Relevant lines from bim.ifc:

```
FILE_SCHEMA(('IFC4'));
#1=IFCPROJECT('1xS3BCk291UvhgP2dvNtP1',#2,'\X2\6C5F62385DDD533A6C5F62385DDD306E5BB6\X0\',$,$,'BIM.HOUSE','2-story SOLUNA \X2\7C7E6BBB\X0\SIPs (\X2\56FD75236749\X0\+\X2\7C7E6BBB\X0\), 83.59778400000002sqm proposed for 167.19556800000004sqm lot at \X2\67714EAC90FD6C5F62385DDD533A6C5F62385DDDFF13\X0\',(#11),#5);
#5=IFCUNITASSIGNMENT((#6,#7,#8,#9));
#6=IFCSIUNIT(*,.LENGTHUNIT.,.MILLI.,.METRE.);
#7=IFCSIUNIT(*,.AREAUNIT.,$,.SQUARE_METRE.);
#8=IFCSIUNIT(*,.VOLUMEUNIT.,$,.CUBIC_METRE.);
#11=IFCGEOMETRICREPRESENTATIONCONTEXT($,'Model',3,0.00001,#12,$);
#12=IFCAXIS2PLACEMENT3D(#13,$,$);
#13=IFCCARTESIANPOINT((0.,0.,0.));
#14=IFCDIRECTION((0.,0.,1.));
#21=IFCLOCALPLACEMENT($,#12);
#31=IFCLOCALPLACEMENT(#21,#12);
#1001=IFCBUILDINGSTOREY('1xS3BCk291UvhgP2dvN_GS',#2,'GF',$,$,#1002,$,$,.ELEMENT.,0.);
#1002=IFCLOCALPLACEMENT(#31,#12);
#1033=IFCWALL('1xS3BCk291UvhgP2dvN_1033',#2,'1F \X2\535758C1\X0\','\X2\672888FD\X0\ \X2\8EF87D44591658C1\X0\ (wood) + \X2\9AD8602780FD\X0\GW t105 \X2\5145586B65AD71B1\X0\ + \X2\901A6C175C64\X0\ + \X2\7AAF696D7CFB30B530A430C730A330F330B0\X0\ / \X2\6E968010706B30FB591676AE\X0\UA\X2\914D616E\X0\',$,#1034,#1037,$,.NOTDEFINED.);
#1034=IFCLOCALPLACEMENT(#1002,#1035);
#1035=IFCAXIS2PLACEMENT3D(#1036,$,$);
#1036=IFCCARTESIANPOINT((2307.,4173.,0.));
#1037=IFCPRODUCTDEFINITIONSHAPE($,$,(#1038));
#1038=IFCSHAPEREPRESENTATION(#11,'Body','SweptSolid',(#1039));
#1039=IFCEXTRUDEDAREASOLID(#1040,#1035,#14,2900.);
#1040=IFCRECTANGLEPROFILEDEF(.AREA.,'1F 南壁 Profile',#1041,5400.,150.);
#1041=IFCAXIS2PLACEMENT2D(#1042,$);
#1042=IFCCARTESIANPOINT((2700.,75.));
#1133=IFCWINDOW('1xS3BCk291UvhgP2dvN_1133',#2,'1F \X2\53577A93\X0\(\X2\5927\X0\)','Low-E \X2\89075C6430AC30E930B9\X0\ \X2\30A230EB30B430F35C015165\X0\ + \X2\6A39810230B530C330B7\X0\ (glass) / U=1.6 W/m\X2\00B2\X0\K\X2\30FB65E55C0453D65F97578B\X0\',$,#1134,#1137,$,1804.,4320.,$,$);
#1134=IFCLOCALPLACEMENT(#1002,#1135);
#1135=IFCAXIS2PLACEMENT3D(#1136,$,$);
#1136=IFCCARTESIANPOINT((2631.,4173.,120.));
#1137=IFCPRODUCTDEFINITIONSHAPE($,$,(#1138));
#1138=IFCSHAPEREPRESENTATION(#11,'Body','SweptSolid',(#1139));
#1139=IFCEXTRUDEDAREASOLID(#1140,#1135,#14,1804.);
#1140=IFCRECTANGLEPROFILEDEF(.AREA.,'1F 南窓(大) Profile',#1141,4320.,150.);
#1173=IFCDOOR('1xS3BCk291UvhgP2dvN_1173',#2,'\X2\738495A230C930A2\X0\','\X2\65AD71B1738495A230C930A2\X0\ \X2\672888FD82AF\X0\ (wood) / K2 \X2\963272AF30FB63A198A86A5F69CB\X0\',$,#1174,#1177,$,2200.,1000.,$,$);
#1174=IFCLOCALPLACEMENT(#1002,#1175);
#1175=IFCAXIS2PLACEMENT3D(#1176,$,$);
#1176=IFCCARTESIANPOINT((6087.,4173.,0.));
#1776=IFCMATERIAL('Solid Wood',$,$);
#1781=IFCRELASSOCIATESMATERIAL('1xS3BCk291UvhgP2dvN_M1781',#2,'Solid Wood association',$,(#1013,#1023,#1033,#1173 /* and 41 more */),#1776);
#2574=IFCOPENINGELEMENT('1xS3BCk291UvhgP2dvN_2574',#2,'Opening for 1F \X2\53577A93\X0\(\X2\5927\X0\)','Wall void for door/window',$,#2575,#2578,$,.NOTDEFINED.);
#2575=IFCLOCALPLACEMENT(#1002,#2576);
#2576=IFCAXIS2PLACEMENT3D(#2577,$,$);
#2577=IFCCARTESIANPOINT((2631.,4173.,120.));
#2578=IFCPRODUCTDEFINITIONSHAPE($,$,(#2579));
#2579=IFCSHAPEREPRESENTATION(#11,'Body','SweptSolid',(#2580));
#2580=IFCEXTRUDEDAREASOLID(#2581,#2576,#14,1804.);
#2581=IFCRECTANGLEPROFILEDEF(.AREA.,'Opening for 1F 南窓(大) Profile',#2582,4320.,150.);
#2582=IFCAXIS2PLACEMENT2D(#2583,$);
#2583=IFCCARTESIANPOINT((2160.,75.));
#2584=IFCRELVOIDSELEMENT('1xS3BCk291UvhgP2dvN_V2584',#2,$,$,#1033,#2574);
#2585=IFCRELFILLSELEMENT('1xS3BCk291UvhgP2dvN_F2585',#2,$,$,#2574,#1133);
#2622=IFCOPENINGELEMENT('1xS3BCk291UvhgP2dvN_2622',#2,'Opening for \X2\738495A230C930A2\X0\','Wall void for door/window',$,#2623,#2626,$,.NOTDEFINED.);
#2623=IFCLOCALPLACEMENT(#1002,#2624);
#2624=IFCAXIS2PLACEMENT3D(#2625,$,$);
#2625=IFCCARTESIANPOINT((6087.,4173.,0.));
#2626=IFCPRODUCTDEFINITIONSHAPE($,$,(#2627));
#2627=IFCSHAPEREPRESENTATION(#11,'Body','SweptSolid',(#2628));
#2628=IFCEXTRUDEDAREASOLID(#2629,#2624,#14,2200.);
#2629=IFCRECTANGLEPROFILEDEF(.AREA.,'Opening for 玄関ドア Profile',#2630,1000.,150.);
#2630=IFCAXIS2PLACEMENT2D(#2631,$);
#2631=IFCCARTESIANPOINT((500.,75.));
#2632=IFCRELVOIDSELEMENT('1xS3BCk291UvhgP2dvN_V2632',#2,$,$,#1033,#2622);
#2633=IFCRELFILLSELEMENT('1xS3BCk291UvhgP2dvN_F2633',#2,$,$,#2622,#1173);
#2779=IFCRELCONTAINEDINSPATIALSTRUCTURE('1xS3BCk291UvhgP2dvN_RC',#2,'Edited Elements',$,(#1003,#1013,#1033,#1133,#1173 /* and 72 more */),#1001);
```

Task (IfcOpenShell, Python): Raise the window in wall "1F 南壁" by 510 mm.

```python
import numpy as np
import ifcopenshell
import ifcopenshell.api.geometry
import ifcopenshell.util.placement
import ifcopenshell.util.unit

model = ifcopenshell.open("bim.ifc")
unit_scale = ifcopenshell.util.unit.calculate_unit_scale(model)

window = model.by_guid("1xS3BCk291UvhgP2dvN_1133")
opening = window.FillsVoids[0].RelatingOpeningElement
dz = 0.51 / unit_scale

shift = np.array([0.0, 0.0, dz])
# The window is not placed relative to its opening, so move both.
for product in (opening, window):
    matrix = ifcopenshell.util.placement.get_local_placement(product.ObjectPlacement)
    matrix[:3, 3] += shift
    ifcopenshell.api.geometry.edit_object_placement(model, product=product, matrix=matrix, is_si=False)

print(f"moved by {dz * unit_scale:+.3f} m")

model.write("bim_edited.ifc")
```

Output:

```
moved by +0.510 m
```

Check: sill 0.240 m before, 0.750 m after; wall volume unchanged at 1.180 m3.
